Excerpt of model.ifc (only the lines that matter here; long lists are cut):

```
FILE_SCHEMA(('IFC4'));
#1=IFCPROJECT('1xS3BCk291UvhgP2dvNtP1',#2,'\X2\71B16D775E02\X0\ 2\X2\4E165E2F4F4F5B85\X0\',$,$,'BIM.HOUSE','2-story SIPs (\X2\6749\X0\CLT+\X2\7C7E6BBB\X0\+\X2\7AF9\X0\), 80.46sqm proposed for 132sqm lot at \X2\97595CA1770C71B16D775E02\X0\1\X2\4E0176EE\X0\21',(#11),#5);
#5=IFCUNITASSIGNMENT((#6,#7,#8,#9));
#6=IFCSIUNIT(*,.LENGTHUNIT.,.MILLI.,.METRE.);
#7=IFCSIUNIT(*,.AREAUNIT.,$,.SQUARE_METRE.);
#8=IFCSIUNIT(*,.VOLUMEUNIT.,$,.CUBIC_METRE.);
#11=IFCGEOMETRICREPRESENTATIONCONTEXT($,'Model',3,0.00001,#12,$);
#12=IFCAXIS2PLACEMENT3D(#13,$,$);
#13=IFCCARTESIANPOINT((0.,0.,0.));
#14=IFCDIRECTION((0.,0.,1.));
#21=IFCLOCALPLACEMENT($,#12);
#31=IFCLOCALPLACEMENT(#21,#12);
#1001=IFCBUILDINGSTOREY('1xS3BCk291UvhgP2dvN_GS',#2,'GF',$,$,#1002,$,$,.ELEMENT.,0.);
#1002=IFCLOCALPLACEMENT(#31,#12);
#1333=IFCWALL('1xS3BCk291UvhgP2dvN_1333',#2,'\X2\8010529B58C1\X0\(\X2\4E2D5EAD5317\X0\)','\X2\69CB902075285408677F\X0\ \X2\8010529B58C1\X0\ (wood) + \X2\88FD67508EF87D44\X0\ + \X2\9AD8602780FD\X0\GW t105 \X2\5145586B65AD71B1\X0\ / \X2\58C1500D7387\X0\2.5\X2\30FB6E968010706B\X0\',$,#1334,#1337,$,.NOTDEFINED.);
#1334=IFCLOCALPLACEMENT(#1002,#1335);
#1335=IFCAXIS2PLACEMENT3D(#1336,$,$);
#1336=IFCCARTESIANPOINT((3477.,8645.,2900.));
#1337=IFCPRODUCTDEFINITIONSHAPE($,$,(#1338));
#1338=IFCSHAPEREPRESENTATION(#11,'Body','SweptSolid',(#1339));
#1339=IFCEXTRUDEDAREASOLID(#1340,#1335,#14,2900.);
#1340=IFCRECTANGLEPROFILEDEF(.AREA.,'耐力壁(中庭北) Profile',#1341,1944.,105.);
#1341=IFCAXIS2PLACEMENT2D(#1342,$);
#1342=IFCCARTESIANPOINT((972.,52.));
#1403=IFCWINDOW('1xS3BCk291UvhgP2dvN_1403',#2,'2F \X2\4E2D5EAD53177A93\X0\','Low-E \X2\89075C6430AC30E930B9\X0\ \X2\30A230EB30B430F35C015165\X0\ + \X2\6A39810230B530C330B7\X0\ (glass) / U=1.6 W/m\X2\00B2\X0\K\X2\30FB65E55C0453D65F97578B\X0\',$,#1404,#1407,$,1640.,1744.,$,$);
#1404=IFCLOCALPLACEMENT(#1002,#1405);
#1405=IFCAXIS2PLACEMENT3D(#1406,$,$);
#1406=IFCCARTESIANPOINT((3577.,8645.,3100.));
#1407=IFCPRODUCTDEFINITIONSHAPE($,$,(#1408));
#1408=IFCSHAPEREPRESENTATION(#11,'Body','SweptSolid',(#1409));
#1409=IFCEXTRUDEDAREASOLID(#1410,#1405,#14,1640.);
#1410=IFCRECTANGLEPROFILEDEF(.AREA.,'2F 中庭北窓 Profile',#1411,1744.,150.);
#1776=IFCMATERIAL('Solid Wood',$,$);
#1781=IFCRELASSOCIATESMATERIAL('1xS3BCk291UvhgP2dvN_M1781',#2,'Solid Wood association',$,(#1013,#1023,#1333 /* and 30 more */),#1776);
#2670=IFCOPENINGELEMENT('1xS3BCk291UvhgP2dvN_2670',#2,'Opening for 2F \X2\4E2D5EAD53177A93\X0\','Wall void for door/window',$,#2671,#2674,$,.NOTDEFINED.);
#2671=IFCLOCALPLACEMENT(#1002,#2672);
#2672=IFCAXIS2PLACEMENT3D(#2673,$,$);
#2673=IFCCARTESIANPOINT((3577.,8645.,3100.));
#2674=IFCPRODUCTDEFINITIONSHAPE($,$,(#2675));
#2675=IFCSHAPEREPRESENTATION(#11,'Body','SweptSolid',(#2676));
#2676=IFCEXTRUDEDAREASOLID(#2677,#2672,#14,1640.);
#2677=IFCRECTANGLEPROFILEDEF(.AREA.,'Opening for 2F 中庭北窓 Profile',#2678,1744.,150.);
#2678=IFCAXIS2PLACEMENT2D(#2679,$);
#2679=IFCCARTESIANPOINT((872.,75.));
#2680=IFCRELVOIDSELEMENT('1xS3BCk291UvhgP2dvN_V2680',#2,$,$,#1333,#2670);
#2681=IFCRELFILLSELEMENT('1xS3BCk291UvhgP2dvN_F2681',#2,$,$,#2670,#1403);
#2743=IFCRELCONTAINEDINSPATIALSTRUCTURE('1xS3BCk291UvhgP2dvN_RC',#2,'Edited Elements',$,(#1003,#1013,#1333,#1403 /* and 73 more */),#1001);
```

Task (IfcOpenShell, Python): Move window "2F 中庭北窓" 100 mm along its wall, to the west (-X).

```python
import ifcopenshell
import ifcopenshell.api.geometry
import ifcopenshell.util.placement
import ifcopenshell.util.unit

model = ifcopenshell.open("model.ifc")
unit_scale = ifcopenshell.util.unit.calculate_unit_scale(model)

window = model.by_id(1403)
opening = window.FillsVoids[0].RelatingOpeningElement
wall = opening.VoidsElements[0].RelatingBuildingElement

wall_matrix = ifcopenshell.util.placement.get_local_placement(wall.ObjectPlacement)
shift = wall_matrix[:3, 0] * -0.1 / unit_scale
before = ifcopenshell.util.placement.get_local_placement(window.ObjectPlacement)[:3, 3].copy()

# The window is not placed relative to its opening, so move both.
for product in (opening, window):
    matrix = ifcopenshell.util.placement.get_local_placement(product.ObjectPlacement)
    matrix[:3, 3] += shift
    ifcopenshell.api.geometry.edit_object_placement(model, product=product, matrix=matrix, is_si=False)

after = ifcopenshell.util.placement.get_local_placement(window.ObjectPlacement)[:3, 3]
print("window moved by", (after - before).round(3) + 0.0)

model.write("model_edited.ifc")
```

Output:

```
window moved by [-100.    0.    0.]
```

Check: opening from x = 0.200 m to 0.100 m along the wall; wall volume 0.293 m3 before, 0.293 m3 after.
